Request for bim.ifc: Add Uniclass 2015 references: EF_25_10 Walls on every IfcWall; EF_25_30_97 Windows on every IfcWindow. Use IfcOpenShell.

First a look at what the model holds.

```python
import ifcopenshell

model = ifcopenshell.open("bim.ifc")
print(model.schema)
print("classifications:", [c.Name for c in model.by_type("IfcClassification")])
for ifc_class in ("IfcDoor", "IfcRoof", "IfcStair", "IfcWall", "IfcWindow"):
    print(ifc_class, len(model.by_type(ifc_class)))
```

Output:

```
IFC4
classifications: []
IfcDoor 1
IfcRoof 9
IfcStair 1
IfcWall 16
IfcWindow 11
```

```python
import ifcopenshell
import ifcopenshell.api.classification

model = ifcopenshell.open("bim.ifc")

system = ifcopenshell.api.classification.add_classification(model, classification="Uniclass 2015")

codes = {
    "IfcWall": ("EF_25_10", "Walls"),
    "IfcWindow": ("EF_25_30_97", "Windows"),
}
for ifc_class, (code, name) in codes.items():
    products = model.by_type(ifc_class)
    ifcopenshell.api.classification.add_reference(
        model, products=products, classification=system, identification=code, name=name
    )
    print(code, len(products))

model.write("bim_edited.ifc")
```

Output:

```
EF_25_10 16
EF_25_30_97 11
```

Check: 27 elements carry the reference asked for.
